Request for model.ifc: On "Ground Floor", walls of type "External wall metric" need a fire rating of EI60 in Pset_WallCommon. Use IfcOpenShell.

First a look at what the model holds.

```python
import ifcopenshell
import ifcopenshell.util.element

model = ifcopenshell.open("model.ifc")
print(model.schema)
storey = next(s for s in model.by_type("IfcBuildingStorey") if s.Name == "Ground Floor")
walls = [e for e in ifcopenshell.util.element.get_decomposition(storey) if e.is_a("IfcWall")]
seen = {}
for e in walls:
    element_type = ifcopenshell.util.element.get_type(e)
    key = (element_type.Name if element_type != e and element_type else None, ifcopenshell.util.element.get_pset(e, "Pset_WallCommon", "FireRating"))
    seen[key] = seen.get(key, 0) + 1
for (name, value), count in sorted(seen.items(), key=str):
    print(count, "x", name, "|", value)
```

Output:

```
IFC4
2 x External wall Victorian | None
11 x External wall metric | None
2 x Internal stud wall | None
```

```python
import ifcopenshell
import ifcopenshell.api.pset
import ifcopenshell.util.element

model = ifcopenshell.open("model.ifc")

storey = next(s for s in model.by_type("IfcBuildingStorey") if s.Name == "Ground Floor")
walls = [e for e in ifcopenshell.util.element.get_decomposition(storey) if e.is_a("IfcWall")]

count = 0
for e in walls:
    element_type = ifcopenshell.util.element.get_type(e)
    if element_type in (None, e) or element_type.Name != "External wall metric":
        continue
    # add_pset returns the element's existing set when there is one.
    pset = ifcopenshell.api.pset.add_pset(model, product=e, name="Pset_WallCommon")
    ifcopenshell.api.pset.edit_pset(model, pset=pset, properties={"FireRating": "EI60"})
    count += 1

print(count, "walls updated")

model.write("model_updated.ifc")
```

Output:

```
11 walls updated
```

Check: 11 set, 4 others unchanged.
